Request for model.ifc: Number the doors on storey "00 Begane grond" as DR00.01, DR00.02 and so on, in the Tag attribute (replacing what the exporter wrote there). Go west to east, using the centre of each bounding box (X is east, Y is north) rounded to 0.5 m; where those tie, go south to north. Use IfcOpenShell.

First a look at what the model holds.

```python
import ifcopenshell
import ifcopenshell.util.element
import ifcopenshell.util.placement

model = ifcopenshell.open("model.ifc")
print(model.schema)
storey = next(s for s in model.by_type("IfcBuildingStorey") if s.Name == "00 Begane grond")
doors = [e for e in ifcopenshell.util.element.get_decomposition(storey) if e.is_a("IfcDoor")]
for e in sorted(doors, key=lambda e: e.id()):
    origin = ifcopenshell.util.placement.get_local_placement(e.ObjectPlacement)[:3, 3]
    print(e.id(), e.Tag, e.Name, origin.round(2) + 0.0, sep=" | ")
```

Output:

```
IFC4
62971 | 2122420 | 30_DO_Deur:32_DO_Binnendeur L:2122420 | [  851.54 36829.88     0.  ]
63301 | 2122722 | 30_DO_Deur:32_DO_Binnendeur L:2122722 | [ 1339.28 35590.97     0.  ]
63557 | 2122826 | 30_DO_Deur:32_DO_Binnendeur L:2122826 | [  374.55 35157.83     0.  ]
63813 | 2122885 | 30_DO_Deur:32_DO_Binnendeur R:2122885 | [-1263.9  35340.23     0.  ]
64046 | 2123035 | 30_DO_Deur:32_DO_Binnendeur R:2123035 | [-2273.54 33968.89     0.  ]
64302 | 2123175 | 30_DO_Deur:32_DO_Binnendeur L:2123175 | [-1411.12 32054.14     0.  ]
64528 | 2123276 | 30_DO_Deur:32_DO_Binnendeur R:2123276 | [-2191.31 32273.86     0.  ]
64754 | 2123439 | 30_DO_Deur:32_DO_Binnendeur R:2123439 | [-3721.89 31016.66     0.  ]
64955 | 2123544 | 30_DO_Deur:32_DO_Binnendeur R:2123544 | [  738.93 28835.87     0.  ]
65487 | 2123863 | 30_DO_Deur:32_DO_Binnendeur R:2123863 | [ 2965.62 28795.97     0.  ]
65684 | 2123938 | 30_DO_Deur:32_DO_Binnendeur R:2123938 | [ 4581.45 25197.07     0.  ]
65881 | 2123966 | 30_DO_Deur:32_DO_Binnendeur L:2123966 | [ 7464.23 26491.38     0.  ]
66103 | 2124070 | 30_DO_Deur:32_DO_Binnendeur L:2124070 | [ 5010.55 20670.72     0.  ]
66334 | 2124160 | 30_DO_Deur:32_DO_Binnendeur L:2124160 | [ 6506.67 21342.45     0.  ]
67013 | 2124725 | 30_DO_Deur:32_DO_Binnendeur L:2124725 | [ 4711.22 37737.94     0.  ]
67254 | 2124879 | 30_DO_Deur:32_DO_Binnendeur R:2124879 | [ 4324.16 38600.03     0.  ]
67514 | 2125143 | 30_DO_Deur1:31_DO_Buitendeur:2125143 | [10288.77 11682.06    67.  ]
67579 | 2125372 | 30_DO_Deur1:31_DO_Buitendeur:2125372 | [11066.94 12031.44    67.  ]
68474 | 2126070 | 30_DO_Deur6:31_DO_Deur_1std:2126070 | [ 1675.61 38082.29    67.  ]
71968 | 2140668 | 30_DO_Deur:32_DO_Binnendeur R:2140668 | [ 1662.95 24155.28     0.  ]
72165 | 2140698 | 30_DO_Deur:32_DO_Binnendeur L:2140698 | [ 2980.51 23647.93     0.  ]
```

```python
import ifcopenshell
import ifcopenshell.geom
import ifcopenshell.util.element
import ifcopenshell.util.shape

model = ifcopenshell.open("model.ifc")
settings = ifcopenshell.geom.settings()
settings.set("use-world-coords", True)


def centre(element):
    shape = ifcopenshell.geom.create_shape(settings, element)
    return ifcopenshell.util.shape.get_bbox_centroid(shape.geometry)


storey = next(s for s in model.by_type("IfcBuildingStorey") if s.Name == "00 Begane grond")
doors = [e for e in ifcopenshell.util.element.get_decomposition(storey) if e.is_a("IfcDoor")]

# Insertion points can sit at a corner or the storey origin, so sort by the geometry (in metres).
centres = {e: centre(e) for e in doors}
doors.sort(key=lambda e: (round(centres[e][0] / 0.5), centres[e][1]))

for i, e in enumerate(doors, start=1):
    number = f"DR00.{i:02d}"
    e.Tag = number
    print(e.id(), number)

model.write("model_updated.ifc")
```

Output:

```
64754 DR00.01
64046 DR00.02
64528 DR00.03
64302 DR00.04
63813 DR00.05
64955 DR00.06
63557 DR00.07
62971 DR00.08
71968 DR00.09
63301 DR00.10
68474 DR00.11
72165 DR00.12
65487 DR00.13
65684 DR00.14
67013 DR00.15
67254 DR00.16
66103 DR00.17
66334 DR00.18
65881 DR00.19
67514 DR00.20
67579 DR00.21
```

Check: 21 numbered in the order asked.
